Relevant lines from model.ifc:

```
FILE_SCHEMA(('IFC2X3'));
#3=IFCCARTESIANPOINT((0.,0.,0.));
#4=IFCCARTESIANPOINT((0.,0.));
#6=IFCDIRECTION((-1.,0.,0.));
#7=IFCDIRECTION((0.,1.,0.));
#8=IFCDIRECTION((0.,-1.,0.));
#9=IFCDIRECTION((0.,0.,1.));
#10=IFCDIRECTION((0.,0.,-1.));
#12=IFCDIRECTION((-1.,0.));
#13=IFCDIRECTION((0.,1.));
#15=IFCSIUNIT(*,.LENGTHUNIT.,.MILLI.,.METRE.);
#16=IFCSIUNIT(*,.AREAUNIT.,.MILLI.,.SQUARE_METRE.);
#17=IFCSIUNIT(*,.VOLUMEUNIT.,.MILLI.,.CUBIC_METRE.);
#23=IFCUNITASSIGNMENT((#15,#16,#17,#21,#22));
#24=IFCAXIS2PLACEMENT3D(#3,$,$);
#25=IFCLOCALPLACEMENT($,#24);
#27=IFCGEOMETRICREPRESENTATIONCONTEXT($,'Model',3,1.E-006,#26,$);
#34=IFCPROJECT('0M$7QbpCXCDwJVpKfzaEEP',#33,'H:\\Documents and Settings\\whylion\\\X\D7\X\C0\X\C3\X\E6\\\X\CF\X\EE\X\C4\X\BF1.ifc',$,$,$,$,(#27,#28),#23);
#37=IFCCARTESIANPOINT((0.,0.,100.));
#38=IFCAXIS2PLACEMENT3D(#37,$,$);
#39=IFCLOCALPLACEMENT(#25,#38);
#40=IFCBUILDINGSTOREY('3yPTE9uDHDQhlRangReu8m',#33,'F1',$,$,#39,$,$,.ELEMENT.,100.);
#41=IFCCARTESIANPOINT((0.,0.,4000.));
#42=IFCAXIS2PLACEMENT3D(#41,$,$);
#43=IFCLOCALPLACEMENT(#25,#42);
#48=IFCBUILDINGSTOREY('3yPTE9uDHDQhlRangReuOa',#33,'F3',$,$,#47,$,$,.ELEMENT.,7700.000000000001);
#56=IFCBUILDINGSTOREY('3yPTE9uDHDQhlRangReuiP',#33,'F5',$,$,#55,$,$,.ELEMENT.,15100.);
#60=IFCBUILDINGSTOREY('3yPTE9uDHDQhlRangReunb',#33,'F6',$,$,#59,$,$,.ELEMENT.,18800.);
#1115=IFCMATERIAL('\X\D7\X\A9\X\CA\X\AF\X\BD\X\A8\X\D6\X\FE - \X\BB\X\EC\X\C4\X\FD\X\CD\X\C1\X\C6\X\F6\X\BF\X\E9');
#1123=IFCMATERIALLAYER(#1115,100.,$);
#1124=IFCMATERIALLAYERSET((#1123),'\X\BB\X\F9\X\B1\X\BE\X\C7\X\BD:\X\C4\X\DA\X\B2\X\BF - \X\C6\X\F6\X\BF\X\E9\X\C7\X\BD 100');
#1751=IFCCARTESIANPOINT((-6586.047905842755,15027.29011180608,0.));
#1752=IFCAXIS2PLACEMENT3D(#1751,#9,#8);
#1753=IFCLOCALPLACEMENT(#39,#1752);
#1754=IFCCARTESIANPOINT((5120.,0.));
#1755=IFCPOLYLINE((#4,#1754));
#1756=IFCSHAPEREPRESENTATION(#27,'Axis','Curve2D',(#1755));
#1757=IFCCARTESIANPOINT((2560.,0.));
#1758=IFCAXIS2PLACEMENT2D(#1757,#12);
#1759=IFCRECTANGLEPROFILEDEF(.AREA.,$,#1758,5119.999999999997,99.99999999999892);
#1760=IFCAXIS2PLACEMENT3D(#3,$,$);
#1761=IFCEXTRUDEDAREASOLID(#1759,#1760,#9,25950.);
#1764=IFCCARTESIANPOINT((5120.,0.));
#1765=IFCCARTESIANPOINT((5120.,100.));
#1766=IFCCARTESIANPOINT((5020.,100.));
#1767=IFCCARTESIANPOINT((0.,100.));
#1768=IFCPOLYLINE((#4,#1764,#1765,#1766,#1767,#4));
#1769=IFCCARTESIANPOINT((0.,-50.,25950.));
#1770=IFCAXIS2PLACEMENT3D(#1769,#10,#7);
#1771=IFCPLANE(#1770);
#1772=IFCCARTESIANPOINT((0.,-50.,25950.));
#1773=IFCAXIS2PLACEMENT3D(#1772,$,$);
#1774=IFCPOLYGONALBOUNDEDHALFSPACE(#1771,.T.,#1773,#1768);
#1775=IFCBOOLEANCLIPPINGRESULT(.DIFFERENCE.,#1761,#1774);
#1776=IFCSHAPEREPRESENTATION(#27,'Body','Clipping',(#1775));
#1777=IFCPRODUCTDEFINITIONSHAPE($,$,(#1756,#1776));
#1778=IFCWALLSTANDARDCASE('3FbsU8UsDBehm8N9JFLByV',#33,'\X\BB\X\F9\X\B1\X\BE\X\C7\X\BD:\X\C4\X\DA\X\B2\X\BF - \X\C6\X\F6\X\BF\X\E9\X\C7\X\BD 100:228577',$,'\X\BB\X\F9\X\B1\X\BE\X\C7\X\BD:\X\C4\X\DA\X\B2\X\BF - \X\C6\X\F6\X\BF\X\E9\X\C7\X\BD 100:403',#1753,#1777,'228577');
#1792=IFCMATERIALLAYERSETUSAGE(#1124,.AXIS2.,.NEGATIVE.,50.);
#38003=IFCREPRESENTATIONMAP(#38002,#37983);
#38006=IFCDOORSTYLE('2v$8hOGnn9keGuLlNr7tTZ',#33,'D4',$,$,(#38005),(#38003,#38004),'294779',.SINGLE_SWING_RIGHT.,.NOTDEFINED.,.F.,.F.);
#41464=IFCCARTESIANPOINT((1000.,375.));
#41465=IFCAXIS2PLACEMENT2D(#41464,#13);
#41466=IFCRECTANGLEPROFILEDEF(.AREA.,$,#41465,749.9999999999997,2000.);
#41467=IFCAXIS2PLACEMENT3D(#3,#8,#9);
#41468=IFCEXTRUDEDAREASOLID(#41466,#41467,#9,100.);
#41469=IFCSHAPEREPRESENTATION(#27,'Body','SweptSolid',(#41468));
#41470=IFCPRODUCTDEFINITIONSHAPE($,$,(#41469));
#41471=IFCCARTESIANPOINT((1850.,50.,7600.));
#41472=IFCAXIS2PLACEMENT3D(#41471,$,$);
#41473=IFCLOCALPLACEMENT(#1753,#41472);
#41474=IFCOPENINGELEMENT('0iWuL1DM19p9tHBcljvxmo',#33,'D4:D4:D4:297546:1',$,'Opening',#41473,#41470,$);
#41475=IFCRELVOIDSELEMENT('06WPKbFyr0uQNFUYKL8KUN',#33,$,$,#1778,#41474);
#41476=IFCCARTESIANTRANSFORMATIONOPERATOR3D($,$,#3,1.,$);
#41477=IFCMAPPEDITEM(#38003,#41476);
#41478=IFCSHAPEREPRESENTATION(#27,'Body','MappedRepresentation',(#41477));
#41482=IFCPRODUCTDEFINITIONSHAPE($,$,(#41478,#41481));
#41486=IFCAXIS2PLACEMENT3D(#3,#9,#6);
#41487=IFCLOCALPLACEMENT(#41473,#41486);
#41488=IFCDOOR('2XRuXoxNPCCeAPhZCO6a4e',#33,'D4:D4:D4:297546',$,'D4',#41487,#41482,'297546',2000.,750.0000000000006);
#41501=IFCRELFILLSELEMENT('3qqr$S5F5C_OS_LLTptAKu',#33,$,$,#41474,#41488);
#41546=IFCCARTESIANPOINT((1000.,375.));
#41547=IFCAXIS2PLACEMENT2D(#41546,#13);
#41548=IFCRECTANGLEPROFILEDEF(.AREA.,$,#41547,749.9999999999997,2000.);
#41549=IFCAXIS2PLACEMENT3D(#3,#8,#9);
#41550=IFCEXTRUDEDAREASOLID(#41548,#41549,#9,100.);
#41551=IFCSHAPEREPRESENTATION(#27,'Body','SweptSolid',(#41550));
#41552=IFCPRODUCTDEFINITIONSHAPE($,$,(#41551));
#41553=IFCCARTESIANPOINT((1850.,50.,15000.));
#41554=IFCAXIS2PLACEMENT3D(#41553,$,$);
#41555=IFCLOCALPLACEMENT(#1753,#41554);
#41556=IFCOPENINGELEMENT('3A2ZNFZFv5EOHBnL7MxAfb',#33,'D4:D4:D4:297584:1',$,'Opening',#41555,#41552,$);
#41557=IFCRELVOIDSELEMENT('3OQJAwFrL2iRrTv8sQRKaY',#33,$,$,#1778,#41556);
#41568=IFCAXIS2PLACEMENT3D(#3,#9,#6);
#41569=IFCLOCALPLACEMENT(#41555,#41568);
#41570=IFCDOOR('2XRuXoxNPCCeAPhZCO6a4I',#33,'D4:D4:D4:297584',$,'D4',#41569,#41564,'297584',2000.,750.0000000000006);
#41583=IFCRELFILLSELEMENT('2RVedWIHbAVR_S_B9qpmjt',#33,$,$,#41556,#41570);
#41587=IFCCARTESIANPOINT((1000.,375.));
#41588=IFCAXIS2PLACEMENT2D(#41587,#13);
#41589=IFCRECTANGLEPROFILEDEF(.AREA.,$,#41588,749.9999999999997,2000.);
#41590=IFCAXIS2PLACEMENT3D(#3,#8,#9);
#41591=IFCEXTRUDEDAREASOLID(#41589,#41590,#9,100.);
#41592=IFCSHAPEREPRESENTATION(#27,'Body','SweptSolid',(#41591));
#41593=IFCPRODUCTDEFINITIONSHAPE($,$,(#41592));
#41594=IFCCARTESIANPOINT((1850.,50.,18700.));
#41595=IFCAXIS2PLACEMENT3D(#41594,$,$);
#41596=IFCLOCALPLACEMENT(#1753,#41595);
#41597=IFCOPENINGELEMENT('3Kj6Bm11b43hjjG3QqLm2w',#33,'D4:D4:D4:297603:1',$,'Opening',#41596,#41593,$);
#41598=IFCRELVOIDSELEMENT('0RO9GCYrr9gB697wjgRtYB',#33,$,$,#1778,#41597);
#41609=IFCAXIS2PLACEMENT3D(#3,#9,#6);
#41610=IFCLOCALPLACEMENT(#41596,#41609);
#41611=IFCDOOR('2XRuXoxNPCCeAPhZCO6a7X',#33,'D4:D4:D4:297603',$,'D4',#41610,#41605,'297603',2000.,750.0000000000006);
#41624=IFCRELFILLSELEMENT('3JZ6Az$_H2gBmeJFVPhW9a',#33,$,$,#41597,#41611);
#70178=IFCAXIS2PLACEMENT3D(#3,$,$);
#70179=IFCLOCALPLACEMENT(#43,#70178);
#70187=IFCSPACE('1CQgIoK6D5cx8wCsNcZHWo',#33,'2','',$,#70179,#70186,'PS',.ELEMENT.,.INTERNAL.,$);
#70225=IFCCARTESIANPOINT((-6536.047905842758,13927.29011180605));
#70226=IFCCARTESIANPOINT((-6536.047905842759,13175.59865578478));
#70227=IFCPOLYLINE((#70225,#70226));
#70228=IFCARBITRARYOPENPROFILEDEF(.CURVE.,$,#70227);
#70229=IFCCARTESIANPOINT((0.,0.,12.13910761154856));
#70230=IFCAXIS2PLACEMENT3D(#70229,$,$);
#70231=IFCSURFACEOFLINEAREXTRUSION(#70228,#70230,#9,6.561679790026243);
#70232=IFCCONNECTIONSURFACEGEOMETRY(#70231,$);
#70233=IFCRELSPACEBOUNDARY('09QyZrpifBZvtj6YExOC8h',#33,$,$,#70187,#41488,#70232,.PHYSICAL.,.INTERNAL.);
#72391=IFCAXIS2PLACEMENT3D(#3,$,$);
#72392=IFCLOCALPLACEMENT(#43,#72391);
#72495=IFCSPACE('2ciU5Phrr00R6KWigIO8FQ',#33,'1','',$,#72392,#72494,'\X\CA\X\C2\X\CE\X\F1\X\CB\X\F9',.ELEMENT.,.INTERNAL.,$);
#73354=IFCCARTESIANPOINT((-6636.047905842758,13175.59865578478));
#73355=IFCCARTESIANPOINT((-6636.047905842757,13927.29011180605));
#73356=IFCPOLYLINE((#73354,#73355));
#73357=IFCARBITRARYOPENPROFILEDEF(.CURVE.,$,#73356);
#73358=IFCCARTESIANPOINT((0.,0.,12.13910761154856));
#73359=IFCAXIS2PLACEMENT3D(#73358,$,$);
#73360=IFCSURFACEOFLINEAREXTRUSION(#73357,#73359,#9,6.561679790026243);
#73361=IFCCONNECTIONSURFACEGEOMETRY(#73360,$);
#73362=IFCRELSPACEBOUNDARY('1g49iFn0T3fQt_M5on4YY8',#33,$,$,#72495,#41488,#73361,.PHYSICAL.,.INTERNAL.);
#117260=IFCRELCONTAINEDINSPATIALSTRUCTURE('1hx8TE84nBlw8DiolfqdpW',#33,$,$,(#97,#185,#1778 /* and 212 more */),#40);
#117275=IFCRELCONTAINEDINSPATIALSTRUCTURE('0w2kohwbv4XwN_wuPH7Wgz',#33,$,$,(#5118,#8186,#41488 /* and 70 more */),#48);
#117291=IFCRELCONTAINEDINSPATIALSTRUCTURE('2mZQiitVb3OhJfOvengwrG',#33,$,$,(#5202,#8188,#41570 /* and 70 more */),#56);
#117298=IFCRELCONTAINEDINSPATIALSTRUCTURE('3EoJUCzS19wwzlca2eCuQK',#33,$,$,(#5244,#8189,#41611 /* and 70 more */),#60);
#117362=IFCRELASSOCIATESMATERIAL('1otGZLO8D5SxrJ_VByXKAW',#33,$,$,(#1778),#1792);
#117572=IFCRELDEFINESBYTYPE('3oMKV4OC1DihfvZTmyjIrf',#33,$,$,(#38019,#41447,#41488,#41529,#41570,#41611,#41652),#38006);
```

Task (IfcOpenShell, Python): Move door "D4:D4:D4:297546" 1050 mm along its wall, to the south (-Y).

```python
import numpy as np
import ifcopenshell
import ifcopenshell.api.geometry
import ifcopenshell.util.placement

model = ifcopenshell.open("model.ifc")

door = model.by_guid("2XRuXoxNPCCeAPhZCO6a4e")
opening = door.FillsVoids[0].RelatingOpeningElement
wall = opening.VoidsElements[0].RelatingBuildingElement

wall_matrix = ifcopenshell.util.placement.get_local_placement(wall.ObjectPlacement)
shift = wall_matrix[:3, 0] * 1050.0
before = ifcopenshell.util.placement.get_local_placement(door.ObjectPlacement)[:3, 3].copy()

# The door is placed relative to its opening, so it follows when the opening moves.
matrix = ifcopenshell.util.placement.get_local_placement(opening.ObjectPlacement)
matrix[:3, 3] += shift
ifcopenshell.api.geometry.edit_object_placement(
    model, product=opening, matrix=matrix, is_si=False, should_transform_children=True
)

# Space boundary surfaces are stored in each space's coordinates; move them too.
for rel in door.ProvidesBoundaries:
    if not rel.ConnectionGeometry:
        continue
    surface = rel.ConnectionGeometry.SurfaceOnRelatingElement
    space_matrix = ifcopenshell.util.placement.get_local_placement(rel.RelatingSpace.ObjectPlacement)
    point = np.array(surface.Position.Location.Coordinates) + space_matrix[:3, :3].T @ shift
    surface.Position = model.createIfcAxis2Placement3D(
        model.createIfcCartesianPoint(point.tolist()), surface.Position.Axis, surface.Position.RefDirection
    )

after = ifcopenshell.util.placement.get_local_placement(door.ObjectPlacement)[:3, 3]
print("door moved by", (after - before).round(3) + 0.0)

model.write("model_updated.ifc")
```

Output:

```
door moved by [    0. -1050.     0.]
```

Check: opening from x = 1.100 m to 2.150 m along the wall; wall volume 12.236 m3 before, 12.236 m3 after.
